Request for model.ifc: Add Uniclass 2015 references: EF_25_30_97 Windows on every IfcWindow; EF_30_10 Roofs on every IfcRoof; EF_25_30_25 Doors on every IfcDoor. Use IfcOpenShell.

First a look at what the model holds.

```python
import ifcopenshell

model = ifcopenshell.open("model.ifc")
print(model.schema)
print("classifications:", [c.Name for c in model.by_type("IfcClassification")])
for ifc_class in ("IfcDoor", "IfcRoof", "IfcStair", "IfcWall", "IfcWindow"):
    print(ifc_class, len(model.by_type(ifc_class)))
```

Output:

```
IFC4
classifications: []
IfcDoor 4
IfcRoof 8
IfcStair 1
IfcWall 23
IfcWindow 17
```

```python
import ifcopenshell
import ifcopenshell.api.classification

model = ifcopenshell.open("model.ifc")

system = ifcopenshell.api.classification.add_classification(model, classification="Uniclass 2015")

codes = {
    "IfcWindow": ("EF_25_30_97", "Windows"),
    "IfcRoof": ("EF_30_10", "Roofs"),
    "IfcDoor": ("EF_25_30_25", "Doors"),
}
for ifc_class, (code, name) in codes.items():
    products = model.by_type(ifc_class)
    ifcopenshell.api.classification.add_reference(
        model, products=products, classification=system, identification=code, name=name
    )
    print(code, len(products))

model.write("model_edited.ifc")
```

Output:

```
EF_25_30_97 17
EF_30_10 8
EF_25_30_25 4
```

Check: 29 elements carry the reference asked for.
